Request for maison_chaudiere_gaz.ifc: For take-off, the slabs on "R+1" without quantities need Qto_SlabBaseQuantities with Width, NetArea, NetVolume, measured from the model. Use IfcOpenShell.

First a look at what the model holds.

```python
import ifcopenshell
import ifcopenshell.util.element
import ifcopenshell.util.unit

model = ifcopenshell.open("maison_chaudiere_gaz.ifc")
print(model.schema)
for unit_type in ("LENGTHUNIT", "AREAUNIT", "VOLUMEUNIT"):
    print(unit_type, ifcopenshell.util.unit.calculate_unit_scale(model, unit_type))
storey = next(s for s in model.by_type("IfcBuildingStorey") if s.Name == "R+1")
slabs = [e for e in ifcopenshell.util.element.get_decomposition(storey) if e.is_a("IfcSlab")]
for e in sorted(slabs, key=lambda e: e.id()):
    print(e.id(), e.is_a(), e.Name, list(ifcopenshell.util.element.get_psets(e, qtos_only=True)), sep=" | ")
```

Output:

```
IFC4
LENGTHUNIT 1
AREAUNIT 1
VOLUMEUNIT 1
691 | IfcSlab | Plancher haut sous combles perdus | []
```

```python
import ifcopenshell
import ifcopenshell.api.pset
import ifcopenshell.geom
import ifcopenshell.util.element
import ifcopenshell.util.shape
import ifcopenshell.util.unit

model = ifcopenshell.open("maison_chaudiere_gaz.ifc")
unit_scale = ifcopenshell.util.unit.calculate_unit_scale(model)
area_scale = ifcopenshell.util.unit.calculate_unit_scale(model, "AREAUNIT")
volume_scale = ifcopenshell.util.unit.calculate_unit_scale(model, "VOLUMEUNIT")
settings = ifcopenshell.geom.settings()

storey = next(s for s in model.by_type("IfcBuildingStorey") if s.Name == "R+1")
slabs = [e for e in ifcopenshell.util.element.get_decomposition(storey) if e.is_a("IfcSlab")]

for e in sorted(slabs, key=lambda e: e.id()):
    if ifcopenshell.util.element.get_psets(e, qtos_only=True, should_inherit=False):
        continue
    # Geometry comes back in metres, in the element's own axes.
    shape = ifcopenshell.geom.create_shape(settings, e)
    values = {
        "Width": ifcopenshell.util.shape.get_z(shape.geometry) / unit_scale,
        "NetArea": ifcopenshell.util.shape.get_footprint_area(shape.geometry) / area_scale,
        "NetVolume": ifcopenshell.util.shape.get_volume(shape.geometry) / volume_scale,
    }
    qto = ifcopenshell.api.pset.add_qto(model, product=e, name="Qto_SlabBaseQuantities")
    ifcopenshell.api.pset.edit_qto(model, qto=qto, properties=values)
    print(e.id(), {k: round(v, 3) for k, v in values.items()})

model.write("maison_chaudiere_gaz_updated.ifc")
```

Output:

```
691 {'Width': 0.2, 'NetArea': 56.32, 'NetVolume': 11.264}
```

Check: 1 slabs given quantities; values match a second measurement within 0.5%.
